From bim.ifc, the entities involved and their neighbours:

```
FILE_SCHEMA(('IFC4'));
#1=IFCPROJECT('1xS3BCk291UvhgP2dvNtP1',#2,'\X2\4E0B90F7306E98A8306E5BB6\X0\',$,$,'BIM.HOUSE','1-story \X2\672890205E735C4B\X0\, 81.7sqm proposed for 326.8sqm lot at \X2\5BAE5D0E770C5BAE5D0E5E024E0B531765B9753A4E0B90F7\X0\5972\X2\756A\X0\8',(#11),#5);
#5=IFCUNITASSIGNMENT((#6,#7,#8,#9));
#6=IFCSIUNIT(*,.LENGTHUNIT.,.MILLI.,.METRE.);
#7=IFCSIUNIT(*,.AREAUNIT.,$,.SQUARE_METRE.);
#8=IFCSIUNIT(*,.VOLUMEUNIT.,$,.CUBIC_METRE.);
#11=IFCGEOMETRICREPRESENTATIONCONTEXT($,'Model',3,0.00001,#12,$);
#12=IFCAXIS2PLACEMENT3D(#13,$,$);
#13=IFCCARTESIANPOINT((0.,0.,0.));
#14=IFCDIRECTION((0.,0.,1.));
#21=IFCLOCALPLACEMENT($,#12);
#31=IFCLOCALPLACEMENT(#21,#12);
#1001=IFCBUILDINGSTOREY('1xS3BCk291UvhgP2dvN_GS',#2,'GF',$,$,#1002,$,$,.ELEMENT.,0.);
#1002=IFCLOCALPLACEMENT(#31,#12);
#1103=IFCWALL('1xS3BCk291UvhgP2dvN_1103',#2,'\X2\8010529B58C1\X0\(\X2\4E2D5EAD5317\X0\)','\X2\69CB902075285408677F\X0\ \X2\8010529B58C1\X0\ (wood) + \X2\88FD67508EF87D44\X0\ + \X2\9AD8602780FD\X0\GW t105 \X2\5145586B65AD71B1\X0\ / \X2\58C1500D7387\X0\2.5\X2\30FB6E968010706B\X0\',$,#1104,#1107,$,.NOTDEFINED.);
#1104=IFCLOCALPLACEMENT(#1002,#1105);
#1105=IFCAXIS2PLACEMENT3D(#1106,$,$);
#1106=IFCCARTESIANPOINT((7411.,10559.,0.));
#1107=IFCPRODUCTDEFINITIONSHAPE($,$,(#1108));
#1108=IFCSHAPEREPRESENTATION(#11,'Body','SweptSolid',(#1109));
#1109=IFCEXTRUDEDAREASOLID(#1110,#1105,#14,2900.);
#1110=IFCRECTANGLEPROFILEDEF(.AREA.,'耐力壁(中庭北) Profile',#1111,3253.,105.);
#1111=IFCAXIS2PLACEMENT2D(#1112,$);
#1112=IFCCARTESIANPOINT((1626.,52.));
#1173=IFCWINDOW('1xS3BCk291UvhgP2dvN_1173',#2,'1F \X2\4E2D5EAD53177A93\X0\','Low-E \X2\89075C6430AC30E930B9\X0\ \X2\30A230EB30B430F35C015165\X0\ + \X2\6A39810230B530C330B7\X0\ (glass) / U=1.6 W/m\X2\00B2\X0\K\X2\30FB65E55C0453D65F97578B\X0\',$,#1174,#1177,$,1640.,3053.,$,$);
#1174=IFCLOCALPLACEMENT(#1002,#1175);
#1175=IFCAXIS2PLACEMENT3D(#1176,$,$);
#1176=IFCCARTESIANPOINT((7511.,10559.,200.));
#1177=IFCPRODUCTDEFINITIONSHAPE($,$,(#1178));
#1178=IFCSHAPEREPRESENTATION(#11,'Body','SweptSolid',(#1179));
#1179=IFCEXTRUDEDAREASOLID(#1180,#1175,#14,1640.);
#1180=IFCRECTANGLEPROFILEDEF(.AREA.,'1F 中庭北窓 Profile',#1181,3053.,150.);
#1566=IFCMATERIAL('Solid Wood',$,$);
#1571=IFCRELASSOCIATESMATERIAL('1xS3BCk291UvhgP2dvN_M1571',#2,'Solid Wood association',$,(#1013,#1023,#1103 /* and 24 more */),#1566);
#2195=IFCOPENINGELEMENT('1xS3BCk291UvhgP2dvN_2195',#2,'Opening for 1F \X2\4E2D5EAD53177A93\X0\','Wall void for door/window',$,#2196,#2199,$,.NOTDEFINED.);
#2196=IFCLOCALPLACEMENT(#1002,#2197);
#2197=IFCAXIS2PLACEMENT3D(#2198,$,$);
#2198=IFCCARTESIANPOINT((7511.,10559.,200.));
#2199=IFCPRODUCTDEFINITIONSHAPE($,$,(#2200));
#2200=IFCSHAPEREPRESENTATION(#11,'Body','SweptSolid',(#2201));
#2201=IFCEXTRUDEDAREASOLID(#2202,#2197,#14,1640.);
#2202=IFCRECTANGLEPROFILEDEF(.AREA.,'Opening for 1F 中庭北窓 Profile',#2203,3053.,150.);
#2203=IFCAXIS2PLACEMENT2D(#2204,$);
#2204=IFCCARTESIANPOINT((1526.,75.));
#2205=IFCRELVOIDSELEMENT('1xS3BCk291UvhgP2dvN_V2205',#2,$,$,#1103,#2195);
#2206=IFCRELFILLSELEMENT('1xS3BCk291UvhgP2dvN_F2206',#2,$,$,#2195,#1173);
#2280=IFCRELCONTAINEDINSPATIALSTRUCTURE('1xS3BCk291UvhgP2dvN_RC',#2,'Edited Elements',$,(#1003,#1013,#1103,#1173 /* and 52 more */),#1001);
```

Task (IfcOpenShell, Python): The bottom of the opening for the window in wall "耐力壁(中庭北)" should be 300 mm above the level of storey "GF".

```python
import numpy as np
import ifcopenshell
import ifcopenshell.api.geometry
import ifcopenshell.geom
import ifcopenshell.util.element
import ifcopenshell.util.placement
import ifcopenshell.util.shape
import ifcopenshell.util.unit

model = ifcopenshell.open("bim.ifc")
unit_scale = ifcopenshell.util.unit.calculate_unit_scale(model)

window = model.by_guid("1xS3BCk291UvhgP2dvN_1173")
opening = window.FillsVoids[0].RelatingOpeningElement
storey = ifcopenshell.util.element.get_container(window, ifc_class="IfcBuildingStorey")
level = ifcopenshell.util.placement.get_local_placement(storey.ObjectPlacement)[2, 3]

# The opening's origin need not be at the sill, so measure its lowest point.
shape = ifcopenshell.geom.create_shape(ifcopenshell.geom.settings(), opening)
bottom = ifcopenshell.util.shape.get_shape_bottom_elevation(shape, shape.geometry) / unit_scale
dz = level + 0.3 / unit_scale - bottom

shift = np.array([0.0, 0.0, dz])
# The window is not placed relative to its opening, so move both.
for product in (opening, window):
    matrix = ifcopenshell.util.placement.get_local_placement(product.ObjectPlacement)
    matrix[:3, 3] += shift
    ifcopenshell.api.geometry.edit_object_placement(model, product=product, matrix=matrix, is_si=False)

print(f"moved by {dz * unit_scale:+.3f} m")

model.write("bim_v2.ifc")
```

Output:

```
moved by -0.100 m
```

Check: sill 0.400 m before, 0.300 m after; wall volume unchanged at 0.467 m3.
